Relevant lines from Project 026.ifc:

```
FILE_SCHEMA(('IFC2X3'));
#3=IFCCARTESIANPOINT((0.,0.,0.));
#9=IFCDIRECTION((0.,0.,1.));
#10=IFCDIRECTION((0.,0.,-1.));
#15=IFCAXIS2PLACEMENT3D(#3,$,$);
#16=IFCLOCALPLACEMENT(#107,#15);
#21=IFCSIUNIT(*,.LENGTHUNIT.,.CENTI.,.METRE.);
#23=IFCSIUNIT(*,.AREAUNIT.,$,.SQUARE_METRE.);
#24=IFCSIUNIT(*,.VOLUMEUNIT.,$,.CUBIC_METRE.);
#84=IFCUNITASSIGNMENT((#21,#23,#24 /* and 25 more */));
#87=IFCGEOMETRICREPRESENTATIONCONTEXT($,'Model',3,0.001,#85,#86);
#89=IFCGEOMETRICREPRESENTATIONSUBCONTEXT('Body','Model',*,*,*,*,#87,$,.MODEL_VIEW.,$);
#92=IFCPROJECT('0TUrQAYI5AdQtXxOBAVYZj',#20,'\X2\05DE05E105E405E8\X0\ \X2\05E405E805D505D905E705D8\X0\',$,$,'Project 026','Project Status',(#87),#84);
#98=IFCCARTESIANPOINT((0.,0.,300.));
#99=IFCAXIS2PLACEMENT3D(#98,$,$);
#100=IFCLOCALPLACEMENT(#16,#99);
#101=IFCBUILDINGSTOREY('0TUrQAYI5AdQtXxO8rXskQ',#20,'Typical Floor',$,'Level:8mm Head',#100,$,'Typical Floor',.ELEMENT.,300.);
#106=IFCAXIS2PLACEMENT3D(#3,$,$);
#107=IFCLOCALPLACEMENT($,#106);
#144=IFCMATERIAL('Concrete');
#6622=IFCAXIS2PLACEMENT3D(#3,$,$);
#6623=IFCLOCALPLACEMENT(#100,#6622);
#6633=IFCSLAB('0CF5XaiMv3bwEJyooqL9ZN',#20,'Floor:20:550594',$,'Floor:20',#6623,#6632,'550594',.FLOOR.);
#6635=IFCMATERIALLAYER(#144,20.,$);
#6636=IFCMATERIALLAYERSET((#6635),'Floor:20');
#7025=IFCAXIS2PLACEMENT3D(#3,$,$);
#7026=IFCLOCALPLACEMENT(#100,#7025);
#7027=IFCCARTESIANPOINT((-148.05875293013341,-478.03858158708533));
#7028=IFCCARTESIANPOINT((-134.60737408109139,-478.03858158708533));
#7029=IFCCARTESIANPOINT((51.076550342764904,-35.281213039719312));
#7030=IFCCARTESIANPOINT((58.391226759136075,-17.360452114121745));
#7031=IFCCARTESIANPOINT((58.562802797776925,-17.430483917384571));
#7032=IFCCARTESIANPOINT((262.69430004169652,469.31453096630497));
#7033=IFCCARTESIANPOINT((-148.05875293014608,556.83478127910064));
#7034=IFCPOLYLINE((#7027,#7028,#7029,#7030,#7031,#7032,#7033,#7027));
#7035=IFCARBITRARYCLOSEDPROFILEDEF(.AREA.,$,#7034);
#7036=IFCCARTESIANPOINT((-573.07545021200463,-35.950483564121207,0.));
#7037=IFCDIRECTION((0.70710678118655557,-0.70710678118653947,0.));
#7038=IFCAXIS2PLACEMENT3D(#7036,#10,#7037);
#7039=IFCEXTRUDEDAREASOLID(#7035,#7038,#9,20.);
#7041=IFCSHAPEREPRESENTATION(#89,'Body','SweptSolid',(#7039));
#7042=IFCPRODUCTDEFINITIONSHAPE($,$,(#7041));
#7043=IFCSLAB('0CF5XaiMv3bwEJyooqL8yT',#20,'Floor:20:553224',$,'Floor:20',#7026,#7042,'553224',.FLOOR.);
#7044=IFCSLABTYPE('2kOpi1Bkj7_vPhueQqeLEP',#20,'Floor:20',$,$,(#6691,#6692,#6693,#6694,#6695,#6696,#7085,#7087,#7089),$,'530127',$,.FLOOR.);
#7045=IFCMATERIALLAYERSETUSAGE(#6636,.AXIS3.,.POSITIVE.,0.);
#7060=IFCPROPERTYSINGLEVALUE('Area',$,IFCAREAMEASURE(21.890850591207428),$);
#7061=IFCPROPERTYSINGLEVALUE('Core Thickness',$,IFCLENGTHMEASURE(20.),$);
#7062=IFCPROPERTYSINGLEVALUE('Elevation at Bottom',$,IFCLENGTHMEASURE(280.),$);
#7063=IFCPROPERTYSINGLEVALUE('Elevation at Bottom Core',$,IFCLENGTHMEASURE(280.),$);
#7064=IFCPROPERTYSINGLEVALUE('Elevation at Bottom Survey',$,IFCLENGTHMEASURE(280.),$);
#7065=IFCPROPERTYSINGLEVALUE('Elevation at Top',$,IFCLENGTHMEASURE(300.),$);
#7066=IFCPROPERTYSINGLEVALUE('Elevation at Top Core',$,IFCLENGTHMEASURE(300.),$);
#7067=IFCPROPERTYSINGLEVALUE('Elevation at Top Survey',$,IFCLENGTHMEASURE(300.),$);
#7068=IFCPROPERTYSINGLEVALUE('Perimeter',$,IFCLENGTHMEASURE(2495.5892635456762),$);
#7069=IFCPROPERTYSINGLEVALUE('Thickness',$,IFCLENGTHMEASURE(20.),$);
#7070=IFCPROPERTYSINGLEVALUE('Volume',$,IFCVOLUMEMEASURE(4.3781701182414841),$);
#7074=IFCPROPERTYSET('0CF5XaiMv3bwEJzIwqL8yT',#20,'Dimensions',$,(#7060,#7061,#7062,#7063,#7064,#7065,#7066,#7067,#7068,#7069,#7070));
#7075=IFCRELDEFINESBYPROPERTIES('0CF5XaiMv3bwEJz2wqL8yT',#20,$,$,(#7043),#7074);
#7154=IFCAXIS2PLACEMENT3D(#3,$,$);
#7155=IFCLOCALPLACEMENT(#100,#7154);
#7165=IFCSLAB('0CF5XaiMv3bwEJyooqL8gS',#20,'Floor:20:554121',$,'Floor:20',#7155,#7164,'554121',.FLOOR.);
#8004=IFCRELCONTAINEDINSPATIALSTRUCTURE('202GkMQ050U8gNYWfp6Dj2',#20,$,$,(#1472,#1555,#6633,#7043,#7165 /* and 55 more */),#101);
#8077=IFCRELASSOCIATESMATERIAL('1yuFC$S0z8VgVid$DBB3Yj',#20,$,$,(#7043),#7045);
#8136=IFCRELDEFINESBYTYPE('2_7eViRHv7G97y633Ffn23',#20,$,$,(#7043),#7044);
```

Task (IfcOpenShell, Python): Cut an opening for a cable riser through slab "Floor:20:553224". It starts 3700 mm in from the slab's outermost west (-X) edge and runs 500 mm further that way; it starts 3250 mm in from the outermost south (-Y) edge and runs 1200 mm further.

```python
import numpy as np
import ifcopenshell
import ifcopenshell.api.feature
import ifcopenshell.api.geometry
import ifcopenshell.api.pset
import ifcopenshell.api.root
import ifcopenshell.geom
import ifcopenshell.util.element
import ifcopenshell.util.placement
import ifcopenshell.util.representation
import ifcopenshell.util.shape
import ifcopenshell.util.unit

model = ifcopenshell.open("Project 026.ifc")
unit_scale = ifcopenshell.util.unit.calculate_unit_scale(model)
area_scale = ifcopenshell.util.unit.calculate_unit_scale(model, "AREAUNIT")
volume_scale = ifcopenshell.util.unit.calculate_unit_scale(model, "VOLUMEUNIT")
settings = ifcopenshell.geom.settings()


def volume(element):
    """Net volume in cubic metres, openings subtracted."""
    shape = ifcopenshell.geom.create_shape(settings, element)
    return ifcopenshell.util.shape.get_volume(shape.geometry)


slab = model.by_guid("0CF5XaiMv3bwEJyooqL8yT")
before = volume(slab)

# Extent in the slab's own axes, in metres. The edges named are its -X and -Y sides.
slab_shape = ifcopenshell.geom.create_shape(settings, slab)
vertices = ifcopenshell.util.shape.get_vertices(slab_shape.geometry)
x_min, y_min, bottom = vertices.min(axis=0)
top = vertices[:, 2].max()

opening = ifcopenshell.api.root.create_entity(model, ifc_class="IfcOpeningElement", name="Cable riser opening")
context = ifcopenshell.util.representation.get_context(model, "Model", "Body", "MODEL_VIEW")
width, depth = 0.5, 1.2
outline = [(0.0, 0.0), (width, 0.0), (width, depth), (0.0, depth), (0.0, 0.0)]
# Overshoot both faces by 50 mm so the cut is clean.
shape = ifcopenshell.api.geometry.add_slab_representation(
    model, context=context, depth=top - bottom + 0.1, polyline=outline
)
ifcopenshell.api.geometry.assign_representation(model, product=opening, representation=shape)

matrix = ifcopenshell.util.placement.get_local_placement(slab.ObjectPlacement)
matrix[:, 3] = matrix @ np.append(np.array([x_min + 3.7, y_min + 3.25, bottom - 0.05]) / unit_scale, 1.0)
ifcopenshell.api.geometry.edit_object_placement(model, product=opening, matrix=matrix, is_si=False)
ifcopenshell.api.feature.add_feature(model, feature=opening, element=slab)

after = volume(slab)

# Update the slab's stored quantities.
pset = model.by_id(ifcopenshell.util.element.get_pset(slab, "Dimensions", should_inherit=False)["id"])
ifcopenshell.api.pset.edit_pset(model, pset=pset, properties={
    "Area": model.create_entity("IfcAreaMeasure", after / (top - bottom) / area_scale),
    "Volume": model.create_entity("IfcVolumeMeasure", after / volume_scale),
})

print(f"slab volume {before:.3f} -> {after:.3f} m3")

model.write("Project 026-out.ifc")
```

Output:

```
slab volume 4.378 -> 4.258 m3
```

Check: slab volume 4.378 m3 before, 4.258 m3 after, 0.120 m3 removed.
